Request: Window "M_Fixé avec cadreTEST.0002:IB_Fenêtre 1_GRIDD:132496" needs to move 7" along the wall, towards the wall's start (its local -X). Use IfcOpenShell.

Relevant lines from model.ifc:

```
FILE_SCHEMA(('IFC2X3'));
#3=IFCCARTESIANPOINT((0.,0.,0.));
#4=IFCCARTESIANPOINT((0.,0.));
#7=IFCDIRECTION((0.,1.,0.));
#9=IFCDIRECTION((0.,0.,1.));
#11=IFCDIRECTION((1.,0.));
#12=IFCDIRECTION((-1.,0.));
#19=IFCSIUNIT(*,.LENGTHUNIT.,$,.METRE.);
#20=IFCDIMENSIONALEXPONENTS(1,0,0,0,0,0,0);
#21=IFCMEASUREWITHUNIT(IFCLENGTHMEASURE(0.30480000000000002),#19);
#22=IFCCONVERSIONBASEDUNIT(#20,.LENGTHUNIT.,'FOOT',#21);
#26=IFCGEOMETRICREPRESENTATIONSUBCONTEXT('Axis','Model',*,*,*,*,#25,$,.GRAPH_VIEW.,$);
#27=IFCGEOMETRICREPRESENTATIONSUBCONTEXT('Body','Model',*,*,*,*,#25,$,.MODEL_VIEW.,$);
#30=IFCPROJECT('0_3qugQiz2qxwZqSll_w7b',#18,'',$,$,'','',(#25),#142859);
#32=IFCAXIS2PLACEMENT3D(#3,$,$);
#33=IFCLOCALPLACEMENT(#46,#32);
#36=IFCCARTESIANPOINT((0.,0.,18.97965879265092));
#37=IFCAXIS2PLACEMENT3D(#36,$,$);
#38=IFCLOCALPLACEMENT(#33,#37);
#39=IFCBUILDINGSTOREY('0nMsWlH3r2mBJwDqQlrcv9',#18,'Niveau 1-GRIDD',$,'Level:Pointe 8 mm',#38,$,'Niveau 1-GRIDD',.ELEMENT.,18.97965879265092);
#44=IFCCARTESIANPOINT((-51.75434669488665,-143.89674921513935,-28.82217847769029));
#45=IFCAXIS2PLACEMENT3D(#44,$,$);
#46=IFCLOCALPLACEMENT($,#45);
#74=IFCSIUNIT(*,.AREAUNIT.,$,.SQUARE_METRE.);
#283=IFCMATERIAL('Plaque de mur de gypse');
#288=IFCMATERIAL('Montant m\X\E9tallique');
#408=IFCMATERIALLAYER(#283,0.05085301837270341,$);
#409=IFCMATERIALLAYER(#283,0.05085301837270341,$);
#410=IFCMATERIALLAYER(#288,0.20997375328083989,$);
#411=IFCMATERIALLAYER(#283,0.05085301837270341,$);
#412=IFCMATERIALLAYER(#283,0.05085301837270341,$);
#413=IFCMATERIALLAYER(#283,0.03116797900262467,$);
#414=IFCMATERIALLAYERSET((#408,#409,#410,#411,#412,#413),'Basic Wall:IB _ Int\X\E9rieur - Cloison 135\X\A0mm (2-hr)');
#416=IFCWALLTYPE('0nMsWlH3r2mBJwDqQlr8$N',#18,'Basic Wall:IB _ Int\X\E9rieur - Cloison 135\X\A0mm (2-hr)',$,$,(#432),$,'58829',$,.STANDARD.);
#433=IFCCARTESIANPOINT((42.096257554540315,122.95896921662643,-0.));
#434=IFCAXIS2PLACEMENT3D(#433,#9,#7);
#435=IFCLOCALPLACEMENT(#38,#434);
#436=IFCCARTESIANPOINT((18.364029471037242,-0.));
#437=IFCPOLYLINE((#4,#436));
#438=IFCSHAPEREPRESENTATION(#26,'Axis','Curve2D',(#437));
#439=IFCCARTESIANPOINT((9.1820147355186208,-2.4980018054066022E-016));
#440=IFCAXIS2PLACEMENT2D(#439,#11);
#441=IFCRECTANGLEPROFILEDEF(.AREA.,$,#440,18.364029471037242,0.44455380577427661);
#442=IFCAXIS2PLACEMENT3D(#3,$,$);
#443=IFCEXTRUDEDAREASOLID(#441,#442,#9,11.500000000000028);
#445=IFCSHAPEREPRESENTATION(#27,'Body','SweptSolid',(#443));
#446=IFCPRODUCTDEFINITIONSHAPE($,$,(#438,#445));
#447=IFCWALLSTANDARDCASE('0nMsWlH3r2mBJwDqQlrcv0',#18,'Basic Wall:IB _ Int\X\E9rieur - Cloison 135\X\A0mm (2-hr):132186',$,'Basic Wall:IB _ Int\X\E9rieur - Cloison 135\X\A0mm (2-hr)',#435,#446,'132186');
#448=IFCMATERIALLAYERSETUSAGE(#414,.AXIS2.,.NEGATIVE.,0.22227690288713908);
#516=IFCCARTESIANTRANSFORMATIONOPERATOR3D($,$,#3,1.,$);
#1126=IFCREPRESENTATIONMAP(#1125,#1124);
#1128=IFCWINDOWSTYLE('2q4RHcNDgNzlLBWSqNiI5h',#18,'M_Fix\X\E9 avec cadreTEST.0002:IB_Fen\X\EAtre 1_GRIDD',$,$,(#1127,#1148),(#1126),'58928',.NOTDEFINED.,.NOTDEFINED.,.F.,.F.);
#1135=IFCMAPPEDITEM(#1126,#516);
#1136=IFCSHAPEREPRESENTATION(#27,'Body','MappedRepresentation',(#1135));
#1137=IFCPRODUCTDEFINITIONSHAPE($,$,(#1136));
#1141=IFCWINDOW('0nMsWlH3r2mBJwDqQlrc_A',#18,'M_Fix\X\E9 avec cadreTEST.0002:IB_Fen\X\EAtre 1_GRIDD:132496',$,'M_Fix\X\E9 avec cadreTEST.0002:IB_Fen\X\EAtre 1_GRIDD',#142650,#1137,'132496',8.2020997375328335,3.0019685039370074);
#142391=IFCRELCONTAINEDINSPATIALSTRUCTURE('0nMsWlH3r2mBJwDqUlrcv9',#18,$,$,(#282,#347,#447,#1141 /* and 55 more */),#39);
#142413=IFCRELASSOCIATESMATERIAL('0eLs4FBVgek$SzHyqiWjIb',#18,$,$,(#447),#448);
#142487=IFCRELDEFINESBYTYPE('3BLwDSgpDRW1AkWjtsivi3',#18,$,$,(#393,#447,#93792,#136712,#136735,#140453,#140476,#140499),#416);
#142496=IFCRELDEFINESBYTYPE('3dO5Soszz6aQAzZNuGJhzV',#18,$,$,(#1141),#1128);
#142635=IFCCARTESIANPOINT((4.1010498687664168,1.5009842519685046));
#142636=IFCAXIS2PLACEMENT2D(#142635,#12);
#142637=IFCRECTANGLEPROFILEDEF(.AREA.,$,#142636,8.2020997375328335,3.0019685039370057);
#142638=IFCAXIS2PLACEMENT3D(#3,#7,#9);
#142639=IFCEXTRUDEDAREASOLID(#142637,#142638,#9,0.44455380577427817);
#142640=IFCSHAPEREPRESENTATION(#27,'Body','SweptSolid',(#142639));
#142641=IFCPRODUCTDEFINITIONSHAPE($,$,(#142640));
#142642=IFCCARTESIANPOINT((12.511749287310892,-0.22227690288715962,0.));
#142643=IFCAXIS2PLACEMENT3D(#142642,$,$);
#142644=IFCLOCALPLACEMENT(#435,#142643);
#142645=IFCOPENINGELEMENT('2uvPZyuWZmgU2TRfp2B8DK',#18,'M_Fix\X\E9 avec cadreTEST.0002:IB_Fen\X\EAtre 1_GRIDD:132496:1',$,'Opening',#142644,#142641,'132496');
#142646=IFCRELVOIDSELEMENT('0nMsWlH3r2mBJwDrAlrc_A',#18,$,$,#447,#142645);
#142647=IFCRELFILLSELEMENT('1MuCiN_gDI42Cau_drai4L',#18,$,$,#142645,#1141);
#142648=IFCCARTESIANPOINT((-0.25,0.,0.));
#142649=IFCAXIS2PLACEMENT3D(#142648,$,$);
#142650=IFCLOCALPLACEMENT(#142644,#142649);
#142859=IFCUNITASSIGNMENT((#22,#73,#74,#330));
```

```python
import ifcopenshell
import ifcopenshell.api.geometry
import ifcopenshell.util.placement
import ifcopenshell.util.unit

model = ifcopenshell.open("model.ifc")
unit_scale = ifcopenshell.util.unit.calculate_unit_scale(model)

window = model.by_guid("0nMsWlH3r2mBJwDqQlrc_A")
opening = window.FillsVoids[0].RelatingOpeningElement
wall = opening.VoidsElements[0].RelatingBuildingElement

wall_matrix = ifcopenshell.util.placement.get_local_placement(wall.ObjectPlacement)
shift = wall_matrix[:3, 0] * -7 * 0.0254 / unit_scale
before = ifcopenshell.util.placement.get_local_placement(window.ObjectPlacement)[:3, 3].copy()

# The window is placed relative to its opening, so it follows when the opening moves.
matrix = ifcopenshell.util.placement.get_local_placement(opening.ObjectPlacement)
matrix[:3, 3] += shift
ifcopenshell.api.geometry.edit_object_placement(
    model, product=opening, matrix=matrix, is_si=False, should_transform_children=True
)

after = ifcopenshell.util.placement.get_local_placement(window.ObjectPlacement)[:3, 3]
print("window moved by", (after - before).round(3) + 0.0)

model.write("model_rev.ifc")
```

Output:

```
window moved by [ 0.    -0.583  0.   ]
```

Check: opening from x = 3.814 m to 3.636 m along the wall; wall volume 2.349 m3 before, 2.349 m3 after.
